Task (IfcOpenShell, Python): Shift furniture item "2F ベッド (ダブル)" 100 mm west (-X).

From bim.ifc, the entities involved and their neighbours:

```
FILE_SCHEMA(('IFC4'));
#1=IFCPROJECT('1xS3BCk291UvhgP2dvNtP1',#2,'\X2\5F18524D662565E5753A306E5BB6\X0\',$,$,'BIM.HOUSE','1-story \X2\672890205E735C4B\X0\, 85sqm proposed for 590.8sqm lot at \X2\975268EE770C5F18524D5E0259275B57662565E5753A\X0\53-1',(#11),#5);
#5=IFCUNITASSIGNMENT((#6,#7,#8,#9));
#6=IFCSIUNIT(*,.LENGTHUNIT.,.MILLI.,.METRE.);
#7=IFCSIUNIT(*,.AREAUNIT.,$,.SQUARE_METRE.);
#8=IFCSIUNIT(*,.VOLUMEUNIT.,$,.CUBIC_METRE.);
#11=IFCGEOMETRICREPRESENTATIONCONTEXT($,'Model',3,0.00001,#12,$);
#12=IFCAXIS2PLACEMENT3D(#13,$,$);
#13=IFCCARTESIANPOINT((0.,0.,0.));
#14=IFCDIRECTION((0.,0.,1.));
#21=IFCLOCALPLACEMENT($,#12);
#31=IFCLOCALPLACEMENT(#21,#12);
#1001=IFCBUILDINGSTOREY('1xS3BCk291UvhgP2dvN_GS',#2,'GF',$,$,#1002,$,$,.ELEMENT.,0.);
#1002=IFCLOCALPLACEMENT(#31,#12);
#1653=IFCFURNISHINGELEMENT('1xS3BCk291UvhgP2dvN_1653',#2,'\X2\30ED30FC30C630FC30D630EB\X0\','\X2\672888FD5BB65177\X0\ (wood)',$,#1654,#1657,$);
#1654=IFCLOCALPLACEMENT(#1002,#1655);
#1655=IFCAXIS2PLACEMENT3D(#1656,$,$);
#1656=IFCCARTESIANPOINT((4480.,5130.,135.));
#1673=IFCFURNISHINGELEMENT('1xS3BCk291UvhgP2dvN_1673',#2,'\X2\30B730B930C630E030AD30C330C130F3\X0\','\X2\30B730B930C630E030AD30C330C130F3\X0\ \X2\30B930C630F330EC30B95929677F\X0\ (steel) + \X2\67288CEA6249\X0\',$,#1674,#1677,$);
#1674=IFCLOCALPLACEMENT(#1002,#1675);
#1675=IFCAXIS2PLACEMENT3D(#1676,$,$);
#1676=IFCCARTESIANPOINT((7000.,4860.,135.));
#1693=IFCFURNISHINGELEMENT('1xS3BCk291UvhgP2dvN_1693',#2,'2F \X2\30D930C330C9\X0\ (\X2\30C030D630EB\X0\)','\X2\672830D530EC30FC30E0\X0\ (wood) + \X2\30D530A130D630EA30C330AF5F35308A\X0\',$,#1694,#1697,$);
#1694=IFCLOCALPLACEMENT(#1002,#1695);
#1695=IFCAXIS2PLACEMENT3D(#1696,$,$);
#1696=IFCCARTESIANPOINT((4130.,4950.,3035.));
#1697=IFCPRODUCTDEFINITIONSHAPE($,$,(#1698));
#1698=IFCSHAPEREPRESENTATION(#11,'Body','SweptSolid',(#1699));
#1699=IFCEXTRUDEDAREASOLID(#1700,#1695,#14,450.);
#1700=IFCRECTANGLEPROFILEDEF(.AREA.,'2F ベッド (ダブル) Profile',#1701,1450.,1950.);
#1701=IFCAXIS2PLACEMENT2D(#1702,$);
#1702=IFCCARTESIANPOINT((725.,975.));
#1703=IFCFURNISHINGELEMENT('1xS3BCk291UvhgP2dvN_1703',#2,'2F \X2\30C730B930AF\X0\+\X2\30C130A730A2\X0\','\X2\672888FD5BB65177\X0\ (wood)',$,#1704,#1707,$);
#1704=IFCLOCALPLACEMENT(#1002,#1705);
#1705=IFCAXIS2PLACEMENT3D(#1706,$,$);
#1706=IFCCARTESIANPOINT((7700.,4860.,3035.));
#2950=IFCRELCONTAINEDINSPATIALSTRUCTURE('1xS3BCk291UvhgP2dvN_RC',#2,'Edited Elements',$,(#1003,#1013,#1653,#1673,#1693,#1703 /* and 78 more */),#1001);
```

```python
import ifcopenshell
import ifcopenshell.api.geometry
import ifcopenshell.util.placement
import ifcopenshell.util.unit

model = ifcopenshell.open("bim.ifc")
unit_scale = ifcopenshell.util.unit.calculate_unit_scale(model)

item = model.by_guid("1xS3BCk291UvhgP2dvN_1693")
matrix = ifcopenshell.util.placement.get_local_placement(item.ObjectPlacement)
matrix[0, 3] -= 0.1 / unit_scale
ifcopenshell.api.geometry.edit_object_placement(model, product=item, matrix=matrix, is_si=False)

print(ifcopenshell.util.placement.get_local_placement(item.ObjectPlacement).round(3) + 0.0)

model.write("bim_v2.ifc")
```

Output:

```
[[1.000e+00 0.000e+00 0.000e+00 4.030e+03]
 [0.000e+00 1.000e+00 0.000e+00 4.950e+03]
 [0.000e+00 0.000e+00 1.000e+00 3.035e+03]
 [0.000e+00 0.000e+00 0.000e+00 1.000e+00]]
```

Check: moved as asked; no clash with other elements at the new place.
